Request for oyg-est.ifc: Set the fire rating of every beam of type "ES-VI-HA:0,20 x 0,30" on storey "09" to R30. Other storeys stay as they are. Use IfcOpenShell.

First a look at what the model holds.

```python
import ifcopenshell
import ifcopenshell.util.element

model = ifcopenshell.open("oyg-est.ifc")
print(model.schema)
storey = next(s for s in model.by_type("IfcBuildingStorey") if s.Name == "09")
beams = [e for e in ifcopenshell.util.element.get_decomposition(storey) if e.is_a("IfcBeam")]
seen = {}
for e in beams:
    element_type = ifcopenshell.util.element.get_type(e)
    key = (element_type.Name if element_type != e and element_type else None, ifcopenshell.util.element.get_pset(e, "Pset_BeamCommon", "FireRating"))
    seen[key] = seen.get(key, 0) + 1
for (name, value), count in sorted(seen.items(), key=str):
    print(count, "x", name, "|", value)
```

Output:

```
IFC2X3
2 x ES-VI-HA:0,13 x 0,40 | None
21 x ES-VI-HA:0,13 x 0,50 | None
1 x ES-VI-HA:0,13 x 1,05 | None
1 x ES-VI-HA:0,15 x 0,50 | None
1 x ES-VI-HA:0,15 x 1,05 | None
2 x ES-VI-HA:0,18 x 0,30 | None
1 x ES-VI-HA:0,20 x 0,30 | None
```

```python
import ifcopenshell
import ifcopenshell.api.pset
import ifcopenshell.util.element

model = ifcopenshell.open("oyg-est.ifc")

storey = next(s for s in model.by_type("IfcBuildingStorey") if s.Name == "09")
beams = [e for e in ifcopenshell.util.element.get_decomposition(storey) if e.is_a("IfcBeam")]

count = 0
for e in beams:
    element_type = ifcopenshell.util.element.get_type(e)
    if element_type in (None, e) or element_type.Name != "ES-VI-HA:0,20 x 0,30":
        continue
    # add_pset returns the element's existing set when there is one.
    pset = ifcopenshell.api.pset.add_pset(model, product=e, name="Pset_BeamCommon")
    ifcopenshell.api.pset.edit_pset(model, pset=pset, properties={"FireRating": "R30"})
    count += 1

print(count, "beams updated")

model.write("oyg-est-out.ifc")
```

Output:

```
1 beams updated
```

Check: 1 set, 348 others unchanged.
